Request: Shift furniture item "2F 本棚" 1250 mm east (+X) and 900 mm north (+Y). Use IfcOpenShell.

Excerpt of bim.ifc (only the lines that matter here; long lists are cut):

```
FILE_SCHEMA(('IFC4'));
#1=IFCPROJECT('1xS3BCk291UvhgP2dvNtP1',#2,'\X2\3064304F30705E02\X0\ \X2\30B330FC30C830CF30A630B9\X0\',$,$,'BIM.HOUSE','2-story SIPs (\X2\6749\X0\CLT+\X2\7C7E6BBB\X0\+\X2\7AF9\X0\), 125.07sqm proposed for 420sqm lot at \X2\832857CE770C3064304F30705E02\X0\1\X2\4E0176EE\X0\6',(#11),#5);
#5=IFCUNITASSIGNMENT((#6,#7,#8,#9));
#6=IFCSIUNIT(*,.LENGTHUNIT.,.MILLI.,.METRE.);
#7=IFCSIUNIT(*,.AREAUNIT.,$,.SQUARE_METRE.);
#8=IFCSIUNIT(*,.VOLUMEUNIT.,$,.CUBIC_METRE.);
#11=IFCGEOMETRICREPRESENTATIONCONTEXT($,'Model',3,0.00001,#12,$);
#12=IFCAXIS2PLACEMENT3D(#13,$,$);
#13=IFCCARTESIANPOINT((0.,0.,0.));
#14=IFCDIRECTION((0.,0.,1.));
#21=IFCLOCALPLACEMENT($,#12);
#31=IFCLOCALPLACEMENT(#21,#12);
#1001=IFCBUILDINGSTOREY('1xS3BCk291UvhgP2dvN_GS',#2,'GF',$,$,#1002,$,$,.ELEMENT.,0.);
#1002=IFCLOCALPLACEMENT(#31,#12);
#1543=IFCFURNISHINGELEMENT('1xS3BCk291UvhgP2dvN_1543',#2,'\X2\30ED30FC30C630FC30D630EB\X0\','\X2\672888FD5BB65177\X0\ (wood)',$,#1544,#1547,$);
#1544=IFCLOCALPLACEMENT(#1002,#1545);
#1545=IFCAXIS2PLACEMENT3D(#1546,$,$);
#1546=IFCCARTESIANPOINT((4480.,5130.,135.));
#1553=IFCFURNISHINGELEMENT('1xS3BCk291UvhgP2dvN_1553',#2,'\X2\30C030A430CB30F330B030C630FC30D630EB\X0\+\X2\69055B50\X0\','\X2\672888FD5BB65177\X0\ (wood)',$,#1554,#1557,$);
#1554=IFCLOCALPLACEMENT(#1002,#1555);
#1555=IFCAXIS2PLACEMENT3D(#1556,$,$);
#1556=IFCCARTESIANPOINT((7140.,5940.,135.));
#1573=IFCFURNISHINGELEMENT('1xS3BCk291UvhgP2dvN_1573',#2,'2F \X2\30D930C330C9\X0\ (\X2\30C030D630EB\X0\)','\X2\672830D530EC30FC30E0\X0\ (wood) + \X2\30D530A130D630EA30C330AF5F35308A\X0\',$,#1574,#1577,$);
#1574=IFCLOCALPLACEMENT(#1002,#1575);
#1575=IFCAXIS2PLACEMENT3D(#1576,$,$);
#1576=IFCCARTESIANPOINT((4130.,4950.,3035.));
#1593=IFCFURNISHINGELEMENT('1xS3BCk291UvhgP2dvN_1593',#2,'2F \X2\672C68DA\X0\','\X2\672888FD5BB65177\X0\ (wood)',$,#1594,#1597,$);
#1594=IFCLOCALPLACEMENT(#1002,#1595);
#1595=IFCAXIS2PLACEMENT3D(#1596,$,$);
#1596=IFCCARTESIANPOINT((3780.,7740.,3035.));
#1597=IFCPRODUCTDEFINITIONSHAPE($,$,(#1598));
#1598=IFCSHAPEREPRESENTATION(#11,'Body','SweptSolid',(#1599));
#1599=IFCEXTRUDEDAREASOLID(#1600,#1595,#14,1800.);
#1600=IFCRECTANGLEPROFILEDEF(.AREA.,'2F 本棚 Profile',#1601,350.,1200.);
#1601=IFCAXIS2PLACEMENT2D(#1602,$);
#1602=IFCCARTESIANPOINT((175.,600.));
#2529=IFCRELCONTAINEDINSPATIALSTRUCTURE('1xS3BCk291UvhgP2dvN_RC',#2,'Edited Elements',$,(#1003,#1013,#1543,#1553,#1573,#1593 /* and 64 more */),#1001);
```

```python
import ifcopenshell
import ifcopenshell.api.geometry
import ifcopenshell.util.placement

model = ifcopenshell.open("bim.ifc")

item = model.by_guid("1xS3BCk291UvhgP2dvN_1593")
matrix = ifcopenshell.util.placement.get_local_placement(item.ObjectPlacement)
matrix[0, 3] += 1250.0
matrix[1, 3] += 900.0
ifcopenshell.api.geometry.edit_object_placement(model, product=item, matrix=matrix, is_si=False)

print(ifcopenshell.util.placement.get_local_placement(item.ObjectPlacement).round(3) + 0.0)

model.write("bim_v2.ifc")
```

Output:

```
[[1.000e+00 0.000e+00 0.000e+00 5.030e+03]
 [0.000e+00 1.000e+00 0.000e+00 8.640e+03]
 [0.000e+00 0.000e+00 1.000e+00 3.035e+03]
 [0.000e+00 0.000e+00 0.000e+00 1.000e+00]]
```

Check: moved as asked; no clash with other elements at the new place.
